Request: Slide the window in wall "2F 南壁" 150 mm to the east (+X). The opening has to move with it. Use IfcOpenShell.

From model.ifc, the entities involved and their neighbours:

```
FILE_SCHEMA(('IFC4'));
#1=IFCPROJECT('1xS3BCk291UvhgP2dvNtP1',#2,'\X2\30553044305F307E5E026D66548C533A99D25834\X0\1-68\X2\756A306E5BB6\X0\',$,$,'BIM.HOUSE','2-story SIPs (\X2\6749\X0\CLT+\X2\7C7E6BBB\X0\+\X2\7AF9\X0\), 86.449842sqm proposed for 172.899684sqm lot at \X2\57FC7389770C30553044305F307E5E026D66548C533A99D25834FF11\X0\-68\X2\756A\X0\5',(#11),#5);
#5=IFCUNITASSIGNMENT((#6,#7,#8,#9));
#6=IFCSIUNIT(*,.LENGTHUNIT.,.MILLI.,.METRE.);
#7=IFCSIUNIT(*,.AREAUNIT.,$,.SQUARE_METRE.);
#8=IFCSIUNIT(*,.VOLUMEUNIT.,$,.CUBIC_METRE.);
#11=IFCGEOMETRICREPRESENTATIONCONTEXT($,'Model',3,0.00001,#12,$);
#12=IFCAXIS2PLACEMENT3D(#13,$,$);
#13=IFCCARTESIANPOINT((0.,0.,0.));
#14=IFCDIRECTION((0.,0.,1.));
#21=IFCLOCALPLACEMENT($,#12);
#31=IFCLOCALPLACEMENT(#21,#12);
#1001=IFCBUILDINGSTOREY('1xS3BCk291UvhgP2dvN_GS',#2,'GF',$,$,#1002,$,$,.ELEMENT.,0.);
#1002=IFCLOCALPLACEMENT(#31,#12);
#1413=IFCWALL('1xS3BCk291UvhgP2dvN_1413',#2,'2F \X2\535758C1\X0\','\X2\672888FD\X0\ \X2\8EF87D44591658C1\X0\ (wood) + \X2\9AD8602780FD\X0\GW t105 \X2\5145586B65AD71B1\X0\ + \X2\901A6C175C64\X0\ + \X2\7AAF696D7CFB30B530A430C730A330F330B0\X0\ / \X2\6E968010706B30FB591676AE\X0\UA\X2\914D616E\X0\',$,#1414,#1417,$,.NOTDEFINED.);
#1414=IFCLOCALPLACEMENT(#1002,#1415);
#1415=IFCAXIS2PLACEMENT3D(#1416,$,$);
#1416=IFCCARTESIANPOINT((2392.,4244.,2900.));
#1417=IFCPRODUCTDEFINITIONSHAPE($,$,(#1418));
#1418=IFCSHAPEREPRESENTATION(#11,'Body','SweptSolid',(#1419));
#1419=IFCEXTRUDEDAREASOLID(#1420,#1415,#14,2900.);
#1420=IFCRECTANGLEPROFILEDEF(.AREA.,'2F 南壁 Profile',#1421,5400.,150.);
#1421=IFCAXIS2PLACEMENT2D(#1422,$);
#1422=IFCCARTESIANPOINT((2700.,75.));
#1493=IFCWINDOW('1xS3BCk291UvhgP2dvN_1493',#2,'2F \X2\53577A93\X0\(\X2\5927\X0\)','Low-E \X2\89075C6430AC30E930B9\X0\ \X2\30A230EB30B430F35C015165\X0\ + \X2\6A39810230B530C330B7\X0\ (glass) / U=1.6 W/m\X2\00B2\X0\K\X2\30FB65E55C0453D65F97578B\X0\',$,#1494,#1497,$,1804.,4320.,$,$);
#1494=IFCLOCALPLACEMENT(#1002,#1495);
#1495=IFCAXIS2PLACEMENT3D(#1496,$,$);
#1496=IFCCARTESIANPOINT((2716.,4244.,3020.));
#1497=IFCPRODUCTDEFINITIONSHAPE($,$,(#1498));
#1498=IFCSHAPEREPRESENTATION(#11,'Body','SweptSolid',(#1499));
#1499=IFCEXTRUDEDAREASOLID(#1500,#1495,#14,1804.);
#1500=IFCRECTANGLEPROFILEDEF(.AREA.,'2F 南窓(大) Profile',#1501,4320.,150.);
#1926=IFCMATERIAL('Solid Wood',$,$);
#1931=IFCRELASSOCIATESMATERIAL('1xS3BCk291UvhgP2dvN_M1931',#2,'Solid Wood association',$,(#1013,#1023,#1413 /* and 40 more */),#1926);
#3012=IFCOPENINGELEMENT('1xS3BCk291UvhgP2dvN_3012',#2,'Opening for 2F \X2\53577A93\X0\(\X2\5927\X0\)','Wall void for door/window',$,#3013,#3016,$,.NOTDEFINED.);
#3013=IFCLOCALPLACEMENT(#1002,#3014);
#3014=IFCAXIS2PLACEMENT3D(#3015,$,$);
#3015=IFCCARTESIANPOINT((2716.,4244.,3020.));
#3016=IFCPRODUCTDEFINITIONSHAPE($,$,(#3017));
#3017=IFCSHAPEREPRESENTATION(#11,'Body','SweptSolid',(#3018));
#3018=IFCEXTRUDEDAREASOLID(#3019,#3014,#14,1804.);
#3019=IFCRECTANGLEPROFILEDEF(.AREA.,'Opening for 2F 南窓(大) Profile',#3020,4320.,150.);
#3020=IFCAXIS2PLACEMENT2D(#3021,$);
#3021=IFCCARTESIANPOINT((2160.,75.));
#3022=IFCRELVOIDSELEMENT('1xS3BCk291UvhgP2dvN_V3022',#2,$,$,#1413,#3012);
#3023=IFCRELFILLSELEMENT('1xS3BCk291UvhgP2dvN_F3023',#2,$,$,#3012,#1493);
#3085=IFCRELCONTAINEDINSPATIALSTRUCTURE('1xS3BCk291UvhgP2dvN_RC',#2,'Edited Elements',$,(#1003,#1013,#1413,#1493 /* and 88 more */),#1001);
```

```python
import ifcopenshell
import ifcopenshell.api.geometry
import ifcopenshell.util.placement
import ifcopenshell.util.unit

model = ifcopenshell.open("model.ifc")
unit_scale = ifcopenshell.util.unit.calculate_unit_scale(model)

window = model.by_guid("1xS3BCk291UvhgP2dvN_1493")
opening = window.FillsVoids[0].RelatingOpeningElement
wall = opening.VoidsElements[0].RelatingBuildingElement

wall_matrix = ifcopenshell.util.placement.get_local_placement(wall.ObjectPlacement)
shift = wall_matrix[:3, 0] * 0.15 / unit_scale
before = ifcopenshell.util.placement.get_local_placement(window.ObjectPlacement)[:3, 3].copy()

# The window is not placed relative to its opening, so move both.
for product in (opening, window):
    matrix = ifcopenshell.util.placement.get_local_placement(product.ObjectPlacement)
    matrix[:3, 3] += shift
    ifcopenshell.api.geometry.edit_object_placement(model, product=product, matrix=matrix, is_si=False)

after = ifcopenshell.util.placement.get_local_placement(window.ObjectPlacement)[:3, 3]
print("window moved by", (after - before).round(3) + 0.0)

model.write("model_rev.ifc")
```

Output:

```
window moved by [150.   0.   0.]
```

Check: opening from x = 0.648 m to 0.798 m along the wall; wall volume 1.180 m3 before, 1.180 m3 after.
